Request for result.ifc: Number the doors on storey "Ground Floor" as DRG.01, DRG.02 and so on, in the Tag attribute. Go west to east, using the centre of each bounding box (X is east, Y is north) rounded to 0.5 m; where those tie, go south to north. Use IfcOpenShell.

First a look at what the model holds.

```python
import ifcopenshell
import ifcopenshell.util.element
import ifcopenshell.util.placement

model = ifcopenshell.open("result.ifc")
print(model.schema)
storey = next(s for s in model.by_type("IfcBuildingStorey") if s.Name == "Ground Floor")
doors = [e for e in ifcopenshell.util.element.get_decomposition(storey) if e.is_a("IfcDoor")]
for e in sorted(doors, key=lambda e: e.id()):
    origin = ifcopenshell.util.placement.get_local_placement(e.ObjectPlacement)[:3, 3]
    print(e.id(), e.Tag, e.Name, origin.round(2) + 0.0, sep=" | ")
```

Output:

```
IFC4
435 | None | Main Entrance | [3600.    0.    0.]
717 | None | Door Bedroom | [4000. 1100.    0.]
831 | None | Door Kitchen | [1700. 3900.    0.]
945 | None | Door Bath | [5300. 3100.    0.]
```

```python
import ifcopenshell
import ifcopenshell.geom
import ifcopenshell.util.element
import ifcopenshell.util.shape

model = ifcopenshell.open("result.ifc")
settings = ifcopenshell.geom.settings()
settings.set("use-world-coords", True)


def centre(element):
    shape = ifcopenshell.geom.create_shape(settings, element)
    return ifcopenshell.util.shape.get_bbox_centroid(shape.geometry)


storey = next(s for s in model.by_type("IfcBuildingStorey") if s.Name == "Ground Floor")
doors = [e for e in ifcopenshell.util.element.get_decomposition(storey) if e.is_a("IfcDoor")]

# Insertion points can sit at a corner or the storey origin, so sort by the geometry (in metres).
centres = {e: centre(e) for e in doors}
doors.sort(key=lambda e: (round(centres[e][0] / 0.5), centres[e][1]))

for i, e in enumerate(doors, start=1):
    number = f"DRG.{i:02d}"
    e.Tag = number
    print(e.id(), number)

model.write("result-out.ifc")
```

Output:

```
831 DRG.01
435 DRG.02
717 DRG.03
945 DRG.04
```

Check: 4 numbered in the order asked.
